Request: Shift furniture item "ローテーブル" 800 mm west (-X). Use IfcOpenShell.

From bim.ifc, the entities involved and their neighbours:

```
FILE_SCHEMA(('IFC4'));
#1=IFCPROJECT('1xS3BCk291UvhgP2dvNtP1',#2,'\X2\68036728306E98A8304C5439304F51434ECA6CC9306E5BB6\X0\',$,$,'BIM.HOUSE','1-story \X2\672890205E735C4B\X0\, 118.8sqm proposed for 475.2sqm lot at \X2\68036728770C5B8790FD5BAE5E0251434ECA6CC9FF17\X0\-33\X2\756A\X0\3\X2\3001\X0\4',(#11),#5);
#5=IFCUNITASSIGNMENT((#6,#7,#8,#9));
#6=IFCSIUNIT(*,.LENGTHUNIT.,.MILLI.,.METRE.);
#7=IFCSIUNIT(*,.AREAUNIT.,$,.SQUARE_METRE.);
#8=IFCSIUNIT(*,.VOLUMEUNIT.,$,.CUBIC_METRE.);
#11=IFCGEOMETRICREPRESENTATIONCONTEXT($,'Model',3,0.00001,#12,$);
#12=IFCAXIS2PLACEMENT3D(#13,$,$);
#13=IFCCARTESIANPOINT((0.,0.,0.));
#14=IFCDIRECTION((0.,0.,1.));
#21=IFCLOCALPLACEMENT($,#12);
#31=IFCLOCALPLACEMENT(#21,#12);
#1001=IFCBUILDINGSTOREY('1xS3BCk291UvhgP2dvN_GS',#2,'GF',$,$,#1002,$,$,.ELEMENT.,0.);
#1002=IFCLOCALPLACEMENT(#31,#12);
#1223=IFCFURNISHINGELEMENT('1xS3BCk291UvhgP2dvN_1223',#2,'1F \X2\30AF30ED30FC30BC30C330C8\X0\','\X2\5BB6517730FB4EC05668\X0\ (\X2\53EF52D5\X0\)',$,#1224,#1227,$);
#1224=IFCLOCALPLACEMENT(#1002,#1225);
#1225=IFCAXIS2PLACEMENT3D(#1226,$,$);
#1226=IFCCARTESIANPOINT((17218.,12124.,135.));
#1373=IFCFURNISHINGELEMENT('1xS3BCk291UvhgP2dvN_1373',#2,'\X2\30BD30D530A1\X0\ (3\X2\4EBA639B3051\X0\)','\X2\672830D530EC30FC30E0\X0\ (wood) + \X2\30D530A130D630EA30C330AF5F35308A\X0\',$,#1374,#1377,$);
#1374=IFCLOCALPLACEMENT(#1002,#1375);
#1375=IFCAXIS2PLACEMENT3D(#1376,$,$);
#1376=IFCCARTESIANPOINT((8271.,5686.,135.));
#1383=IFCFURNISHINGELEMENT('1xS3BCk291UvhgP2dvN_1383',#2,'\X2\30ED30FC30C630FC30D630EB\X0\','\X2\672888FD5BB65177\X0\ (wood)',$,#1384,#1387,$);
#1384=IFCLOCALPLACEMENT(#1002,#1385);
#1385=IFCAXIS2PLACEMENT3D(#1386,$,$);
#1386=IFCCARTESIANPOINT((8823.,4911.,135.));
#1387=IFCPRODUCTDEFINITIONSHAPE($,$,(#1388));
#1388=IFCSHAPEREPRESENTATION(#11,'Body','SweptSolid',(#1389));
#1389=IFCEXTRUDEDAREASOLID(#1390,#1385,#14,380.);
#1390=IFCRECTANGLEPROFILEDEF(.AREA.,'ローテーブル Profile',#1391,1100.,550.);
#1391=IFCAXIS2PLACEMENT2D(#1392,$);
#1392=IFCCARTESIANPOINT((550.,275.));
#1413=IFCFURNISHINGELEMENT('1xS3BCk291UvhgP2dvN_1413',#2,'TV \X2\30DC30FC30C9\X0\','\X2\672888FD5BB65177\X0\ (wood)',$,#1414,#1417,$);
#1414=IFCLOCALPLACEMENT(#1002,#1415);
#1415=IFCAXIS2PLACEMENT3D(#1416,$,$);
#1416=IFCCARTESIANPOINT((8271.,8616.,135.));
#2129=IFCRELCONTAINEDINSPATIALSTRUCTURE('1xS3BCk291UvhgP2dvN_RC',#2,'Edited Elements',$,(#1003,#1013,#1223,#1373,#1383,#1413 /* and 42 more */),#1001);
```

```python
import ifcopenshell
import ifcopenshell.api.geometry
import ifcopenshell.util.placement
import ifcopenshell.util.unit

model = ifcopenshell.open("bim.ifc")
unit_scale = ifcopenshell.util.unit.calculate_unit_scale(model)

item = model.by_guid("1xS3BCk291UvhgP2dvN_1383")
matrix = ifcopenshell.util.placement.get_local_placement(item.ObjectPlacement)
matrix[0, 3] -= 0.8 / unit_scale
ifcopenshell.api.geometry.edit_object_placement(model, product=item, matrix=matrix, is_si=False)

print(ifcopenshell.util.placement.get_local_placement(item.ObjectPlacement).round(3) + 0.0)

model.write("bim-out.ifc")
```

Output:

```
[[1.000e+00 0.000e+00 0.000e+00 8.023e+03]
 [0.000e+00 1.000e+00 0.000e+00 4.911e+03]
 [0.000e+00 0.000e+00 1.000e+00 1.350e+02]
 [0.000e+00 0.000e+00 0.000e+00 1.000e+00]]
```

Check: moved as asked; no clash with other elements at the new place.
